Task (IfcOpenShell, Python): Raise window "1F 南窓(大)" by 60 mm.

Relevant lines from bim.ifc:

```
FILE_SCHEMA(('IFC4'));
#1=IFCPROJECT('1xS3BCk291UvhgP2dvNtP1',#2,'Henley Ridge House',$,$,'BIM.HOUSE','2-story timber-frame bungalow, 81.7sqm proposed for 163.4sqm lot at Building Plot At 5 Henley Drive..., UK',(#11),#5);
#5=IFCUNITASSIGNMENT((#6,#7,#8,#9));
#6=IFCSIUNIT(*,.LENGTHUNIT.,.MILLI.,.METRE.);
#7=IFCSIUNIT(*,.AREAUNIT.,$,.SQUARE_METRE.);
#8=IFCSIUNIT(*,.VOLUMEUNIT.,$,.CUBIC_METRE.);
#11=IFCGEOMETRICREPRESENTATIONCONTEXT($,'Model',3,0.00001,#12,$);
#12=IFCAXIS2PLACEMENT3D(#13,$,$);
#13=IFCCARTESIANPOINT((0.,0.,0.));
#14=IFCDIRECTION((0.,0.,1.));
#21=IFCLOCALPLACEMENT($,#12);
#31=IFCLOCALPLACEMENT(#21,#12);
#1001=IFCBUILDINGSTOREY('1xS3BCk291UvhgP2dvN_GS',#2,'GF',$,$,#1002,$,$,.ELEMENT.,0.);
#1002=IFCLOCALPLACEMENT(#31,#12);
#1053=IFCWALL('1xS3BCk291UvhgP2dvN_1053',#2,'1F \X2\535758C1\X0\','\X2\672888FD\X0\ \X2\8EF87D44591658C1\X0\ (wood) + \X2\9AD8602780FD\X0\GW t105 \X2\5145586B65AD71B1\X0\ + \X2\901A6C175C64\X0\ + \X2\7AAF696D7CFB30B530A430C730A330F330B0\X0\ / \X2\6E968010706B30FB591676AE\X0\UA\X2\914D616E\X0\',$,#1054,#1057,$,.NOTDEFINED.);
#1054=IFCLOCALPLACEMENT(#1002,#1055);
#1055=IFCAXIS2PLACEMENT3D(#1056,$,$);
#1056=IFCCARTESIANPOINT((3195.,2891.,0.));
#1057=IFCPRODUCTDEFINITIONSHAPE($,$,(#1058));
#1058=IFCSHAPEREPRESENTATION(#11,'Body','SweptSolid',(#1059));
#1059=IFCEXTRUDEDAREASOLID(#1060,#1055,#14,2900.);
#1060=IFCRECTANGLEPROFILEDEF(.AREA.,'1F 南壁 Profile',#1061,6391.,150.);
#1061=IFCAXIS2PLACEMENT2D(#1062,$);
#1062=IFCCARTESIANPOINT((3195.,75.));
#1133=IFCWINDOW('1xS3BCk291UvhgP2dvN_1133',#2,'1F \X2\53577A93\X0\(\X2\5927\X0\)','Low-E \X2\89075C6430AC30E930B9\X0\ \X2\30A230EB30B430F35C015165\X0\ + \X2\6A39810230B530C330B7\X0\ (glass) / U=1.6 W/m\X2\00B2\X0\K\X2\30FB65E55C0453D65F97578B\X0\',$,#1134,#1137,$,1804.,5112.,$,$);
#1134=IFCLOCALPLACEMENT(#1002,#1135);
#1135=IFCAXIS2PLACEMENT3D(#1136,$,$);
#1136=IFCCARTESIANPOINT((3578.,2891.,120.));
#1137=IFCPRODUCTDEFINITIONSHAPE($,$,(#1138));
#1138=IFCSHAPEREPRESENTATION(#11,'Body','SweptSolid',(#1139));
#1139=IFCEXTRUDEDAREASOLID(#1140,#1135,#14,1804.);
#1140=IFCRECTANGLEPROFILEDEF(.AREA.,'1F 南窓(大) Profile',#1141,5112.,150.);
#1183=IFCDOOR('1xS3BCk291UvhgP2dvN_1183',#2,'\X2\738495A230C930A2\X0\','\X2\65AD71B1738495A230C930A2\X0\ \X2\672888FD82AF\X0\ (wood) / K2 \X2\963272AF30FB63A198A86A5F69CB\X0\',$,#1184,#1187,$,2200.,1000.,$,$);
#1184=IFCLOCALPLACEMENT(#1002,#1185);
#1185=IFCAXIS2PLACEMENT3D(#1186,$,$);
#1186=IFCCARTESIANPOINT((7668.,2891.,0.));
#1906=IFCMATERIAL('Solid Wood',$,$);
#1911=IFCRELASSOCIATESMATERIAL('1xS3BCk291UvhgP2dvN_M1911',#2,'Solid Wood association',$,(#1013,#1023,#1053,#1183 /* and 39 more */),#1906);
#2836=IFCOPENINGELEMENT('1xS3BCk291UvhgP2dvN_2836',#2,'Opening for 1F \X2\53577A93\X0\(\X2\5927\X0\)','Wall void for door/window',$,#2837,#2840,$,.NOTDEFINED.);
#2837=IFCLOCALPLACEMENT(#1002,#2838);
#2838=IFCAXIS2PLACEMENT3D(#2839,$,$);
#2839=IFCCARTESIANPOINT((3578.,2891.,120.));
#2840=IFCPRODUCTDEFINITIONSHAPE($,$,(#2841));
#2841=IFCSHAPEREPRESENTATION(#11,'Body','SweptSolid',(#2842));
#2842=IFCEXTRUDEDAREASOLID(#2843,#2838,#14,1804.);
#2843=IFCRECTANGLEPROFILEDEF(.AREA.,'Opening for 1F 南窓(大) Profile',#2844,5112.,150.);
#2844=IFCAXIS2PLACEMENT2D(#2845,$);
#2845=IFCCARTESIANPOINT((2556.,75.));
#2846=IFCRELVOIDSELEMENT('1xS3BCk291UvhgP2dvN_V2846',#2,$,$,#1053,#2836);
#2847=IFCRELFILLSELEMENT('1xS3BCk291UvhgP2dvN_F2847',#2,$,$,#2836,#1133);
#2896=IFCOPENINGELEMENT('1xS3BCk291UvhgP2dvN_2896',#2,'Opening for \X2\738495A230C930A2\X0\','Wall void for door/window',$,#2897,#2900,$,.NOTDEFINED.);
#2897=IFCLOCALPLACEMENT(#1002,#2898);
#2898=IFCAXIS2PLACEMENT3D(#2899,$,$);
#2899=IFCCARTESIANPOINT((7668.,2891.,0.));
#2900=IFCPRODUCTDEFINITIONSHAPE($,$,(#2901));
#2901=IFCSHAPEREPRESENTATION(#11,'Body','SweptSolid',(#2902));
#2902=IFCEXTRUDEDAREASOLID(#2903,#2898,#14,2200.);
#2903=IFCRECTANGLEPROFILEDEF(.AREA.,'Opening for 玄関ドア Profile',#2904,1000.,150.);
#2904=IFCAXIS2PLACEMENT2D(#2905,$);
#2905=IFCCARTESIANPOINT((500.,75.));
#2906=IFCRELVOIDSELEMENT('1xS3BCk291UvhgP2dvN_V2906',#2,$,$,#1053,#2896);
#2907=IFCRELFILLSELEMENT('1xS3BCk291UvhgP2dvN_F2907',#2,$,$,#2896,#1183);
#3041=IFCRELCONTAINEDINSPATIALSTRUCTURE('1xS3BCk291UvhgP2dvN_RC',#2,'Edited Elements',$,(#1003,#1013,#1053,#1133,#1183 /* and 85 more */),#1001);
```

```python
import numpy as np
import ifcopenshell
import ifcopenshell.api.geometry
import ifcopenshell.util.placement
import ifcopenshell.util.unit

model = ifcopenshell.open("bim.ifc")
unit_scale = ifcopenshell.util.unit.calculate_unit_scale(model)

window = model.by_guid("1xS3BCk291UvhgP2dvN_1133")
opening = window.FillsVoids[0].RelatingOpeningElement
dz = 60.0

shift = np.array([0.0, 0.0, dz])
# The window is not placed relative to its opening, so move both.
for product in (opening, window):
    matrix = ifcopenshell.util.placement.get_local_placement(product.ObjectPlacement)
    matrix[:3, 3] += shift
    ifcopenshell.api.geometry.edit_object_placement(model, product=product, matrix=matrix, is_si=False)

print(f"moved by {dz * unit_scale:+.3f} m")

model.write("bim-out.ifc")
```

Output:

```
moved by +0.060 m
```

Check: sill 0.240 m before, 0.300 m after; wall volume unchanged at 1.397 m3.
